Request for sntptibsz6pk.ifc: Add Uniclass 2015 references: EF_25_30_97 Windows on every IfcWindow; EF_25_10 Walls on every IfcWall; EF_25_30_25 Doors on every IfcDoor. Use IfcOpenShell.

First a look at what the model holds.

```python
import ifcopenshell

model = ifcopenshell.open("sntptibsz6pk.ifc")
print(model.schema)
print("classifications:", [c.Name for c in model.by_type("IfcClassification")])
for ifc_class in ("IfcDoor", "IfcRoof", "IfcStair", "IfcWall", "IfcWindow"):
    print(ifc_class, len(model.by_type(ifc_class)))
```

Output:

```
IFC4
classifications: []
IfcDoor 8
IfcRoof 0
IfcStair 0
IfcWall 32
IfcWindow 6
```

```python
import ifcopenshell
import ifcopenshell.api.classification

model = ifcopenshell.open("sntptibsz6pk.ifc")

system = ifcopenshell.api.classification.add_classification(model, classification="Uniclass 2015")

codes = {
    "IfcWindow": ("EF_25_30_97", "Windows"),
    "IfcWall": ("EF_25_10", "Walls"),
    "IfcDoor": ("EF_25_30_25", "Doors"),
}
for ifc_class, (code, name) in codes.items():
    products = model.by_type(ifc_class)
    ifcopenshell.api.classification.add_reference(
        model, products=products, classification=system, identification=code, name=name
    )
    print(code, len(products))

model.write("sntptibsz6pk_rev.ifc")
```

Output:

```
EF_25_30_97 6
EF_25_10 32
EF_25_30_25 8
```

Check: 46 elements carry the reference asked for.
